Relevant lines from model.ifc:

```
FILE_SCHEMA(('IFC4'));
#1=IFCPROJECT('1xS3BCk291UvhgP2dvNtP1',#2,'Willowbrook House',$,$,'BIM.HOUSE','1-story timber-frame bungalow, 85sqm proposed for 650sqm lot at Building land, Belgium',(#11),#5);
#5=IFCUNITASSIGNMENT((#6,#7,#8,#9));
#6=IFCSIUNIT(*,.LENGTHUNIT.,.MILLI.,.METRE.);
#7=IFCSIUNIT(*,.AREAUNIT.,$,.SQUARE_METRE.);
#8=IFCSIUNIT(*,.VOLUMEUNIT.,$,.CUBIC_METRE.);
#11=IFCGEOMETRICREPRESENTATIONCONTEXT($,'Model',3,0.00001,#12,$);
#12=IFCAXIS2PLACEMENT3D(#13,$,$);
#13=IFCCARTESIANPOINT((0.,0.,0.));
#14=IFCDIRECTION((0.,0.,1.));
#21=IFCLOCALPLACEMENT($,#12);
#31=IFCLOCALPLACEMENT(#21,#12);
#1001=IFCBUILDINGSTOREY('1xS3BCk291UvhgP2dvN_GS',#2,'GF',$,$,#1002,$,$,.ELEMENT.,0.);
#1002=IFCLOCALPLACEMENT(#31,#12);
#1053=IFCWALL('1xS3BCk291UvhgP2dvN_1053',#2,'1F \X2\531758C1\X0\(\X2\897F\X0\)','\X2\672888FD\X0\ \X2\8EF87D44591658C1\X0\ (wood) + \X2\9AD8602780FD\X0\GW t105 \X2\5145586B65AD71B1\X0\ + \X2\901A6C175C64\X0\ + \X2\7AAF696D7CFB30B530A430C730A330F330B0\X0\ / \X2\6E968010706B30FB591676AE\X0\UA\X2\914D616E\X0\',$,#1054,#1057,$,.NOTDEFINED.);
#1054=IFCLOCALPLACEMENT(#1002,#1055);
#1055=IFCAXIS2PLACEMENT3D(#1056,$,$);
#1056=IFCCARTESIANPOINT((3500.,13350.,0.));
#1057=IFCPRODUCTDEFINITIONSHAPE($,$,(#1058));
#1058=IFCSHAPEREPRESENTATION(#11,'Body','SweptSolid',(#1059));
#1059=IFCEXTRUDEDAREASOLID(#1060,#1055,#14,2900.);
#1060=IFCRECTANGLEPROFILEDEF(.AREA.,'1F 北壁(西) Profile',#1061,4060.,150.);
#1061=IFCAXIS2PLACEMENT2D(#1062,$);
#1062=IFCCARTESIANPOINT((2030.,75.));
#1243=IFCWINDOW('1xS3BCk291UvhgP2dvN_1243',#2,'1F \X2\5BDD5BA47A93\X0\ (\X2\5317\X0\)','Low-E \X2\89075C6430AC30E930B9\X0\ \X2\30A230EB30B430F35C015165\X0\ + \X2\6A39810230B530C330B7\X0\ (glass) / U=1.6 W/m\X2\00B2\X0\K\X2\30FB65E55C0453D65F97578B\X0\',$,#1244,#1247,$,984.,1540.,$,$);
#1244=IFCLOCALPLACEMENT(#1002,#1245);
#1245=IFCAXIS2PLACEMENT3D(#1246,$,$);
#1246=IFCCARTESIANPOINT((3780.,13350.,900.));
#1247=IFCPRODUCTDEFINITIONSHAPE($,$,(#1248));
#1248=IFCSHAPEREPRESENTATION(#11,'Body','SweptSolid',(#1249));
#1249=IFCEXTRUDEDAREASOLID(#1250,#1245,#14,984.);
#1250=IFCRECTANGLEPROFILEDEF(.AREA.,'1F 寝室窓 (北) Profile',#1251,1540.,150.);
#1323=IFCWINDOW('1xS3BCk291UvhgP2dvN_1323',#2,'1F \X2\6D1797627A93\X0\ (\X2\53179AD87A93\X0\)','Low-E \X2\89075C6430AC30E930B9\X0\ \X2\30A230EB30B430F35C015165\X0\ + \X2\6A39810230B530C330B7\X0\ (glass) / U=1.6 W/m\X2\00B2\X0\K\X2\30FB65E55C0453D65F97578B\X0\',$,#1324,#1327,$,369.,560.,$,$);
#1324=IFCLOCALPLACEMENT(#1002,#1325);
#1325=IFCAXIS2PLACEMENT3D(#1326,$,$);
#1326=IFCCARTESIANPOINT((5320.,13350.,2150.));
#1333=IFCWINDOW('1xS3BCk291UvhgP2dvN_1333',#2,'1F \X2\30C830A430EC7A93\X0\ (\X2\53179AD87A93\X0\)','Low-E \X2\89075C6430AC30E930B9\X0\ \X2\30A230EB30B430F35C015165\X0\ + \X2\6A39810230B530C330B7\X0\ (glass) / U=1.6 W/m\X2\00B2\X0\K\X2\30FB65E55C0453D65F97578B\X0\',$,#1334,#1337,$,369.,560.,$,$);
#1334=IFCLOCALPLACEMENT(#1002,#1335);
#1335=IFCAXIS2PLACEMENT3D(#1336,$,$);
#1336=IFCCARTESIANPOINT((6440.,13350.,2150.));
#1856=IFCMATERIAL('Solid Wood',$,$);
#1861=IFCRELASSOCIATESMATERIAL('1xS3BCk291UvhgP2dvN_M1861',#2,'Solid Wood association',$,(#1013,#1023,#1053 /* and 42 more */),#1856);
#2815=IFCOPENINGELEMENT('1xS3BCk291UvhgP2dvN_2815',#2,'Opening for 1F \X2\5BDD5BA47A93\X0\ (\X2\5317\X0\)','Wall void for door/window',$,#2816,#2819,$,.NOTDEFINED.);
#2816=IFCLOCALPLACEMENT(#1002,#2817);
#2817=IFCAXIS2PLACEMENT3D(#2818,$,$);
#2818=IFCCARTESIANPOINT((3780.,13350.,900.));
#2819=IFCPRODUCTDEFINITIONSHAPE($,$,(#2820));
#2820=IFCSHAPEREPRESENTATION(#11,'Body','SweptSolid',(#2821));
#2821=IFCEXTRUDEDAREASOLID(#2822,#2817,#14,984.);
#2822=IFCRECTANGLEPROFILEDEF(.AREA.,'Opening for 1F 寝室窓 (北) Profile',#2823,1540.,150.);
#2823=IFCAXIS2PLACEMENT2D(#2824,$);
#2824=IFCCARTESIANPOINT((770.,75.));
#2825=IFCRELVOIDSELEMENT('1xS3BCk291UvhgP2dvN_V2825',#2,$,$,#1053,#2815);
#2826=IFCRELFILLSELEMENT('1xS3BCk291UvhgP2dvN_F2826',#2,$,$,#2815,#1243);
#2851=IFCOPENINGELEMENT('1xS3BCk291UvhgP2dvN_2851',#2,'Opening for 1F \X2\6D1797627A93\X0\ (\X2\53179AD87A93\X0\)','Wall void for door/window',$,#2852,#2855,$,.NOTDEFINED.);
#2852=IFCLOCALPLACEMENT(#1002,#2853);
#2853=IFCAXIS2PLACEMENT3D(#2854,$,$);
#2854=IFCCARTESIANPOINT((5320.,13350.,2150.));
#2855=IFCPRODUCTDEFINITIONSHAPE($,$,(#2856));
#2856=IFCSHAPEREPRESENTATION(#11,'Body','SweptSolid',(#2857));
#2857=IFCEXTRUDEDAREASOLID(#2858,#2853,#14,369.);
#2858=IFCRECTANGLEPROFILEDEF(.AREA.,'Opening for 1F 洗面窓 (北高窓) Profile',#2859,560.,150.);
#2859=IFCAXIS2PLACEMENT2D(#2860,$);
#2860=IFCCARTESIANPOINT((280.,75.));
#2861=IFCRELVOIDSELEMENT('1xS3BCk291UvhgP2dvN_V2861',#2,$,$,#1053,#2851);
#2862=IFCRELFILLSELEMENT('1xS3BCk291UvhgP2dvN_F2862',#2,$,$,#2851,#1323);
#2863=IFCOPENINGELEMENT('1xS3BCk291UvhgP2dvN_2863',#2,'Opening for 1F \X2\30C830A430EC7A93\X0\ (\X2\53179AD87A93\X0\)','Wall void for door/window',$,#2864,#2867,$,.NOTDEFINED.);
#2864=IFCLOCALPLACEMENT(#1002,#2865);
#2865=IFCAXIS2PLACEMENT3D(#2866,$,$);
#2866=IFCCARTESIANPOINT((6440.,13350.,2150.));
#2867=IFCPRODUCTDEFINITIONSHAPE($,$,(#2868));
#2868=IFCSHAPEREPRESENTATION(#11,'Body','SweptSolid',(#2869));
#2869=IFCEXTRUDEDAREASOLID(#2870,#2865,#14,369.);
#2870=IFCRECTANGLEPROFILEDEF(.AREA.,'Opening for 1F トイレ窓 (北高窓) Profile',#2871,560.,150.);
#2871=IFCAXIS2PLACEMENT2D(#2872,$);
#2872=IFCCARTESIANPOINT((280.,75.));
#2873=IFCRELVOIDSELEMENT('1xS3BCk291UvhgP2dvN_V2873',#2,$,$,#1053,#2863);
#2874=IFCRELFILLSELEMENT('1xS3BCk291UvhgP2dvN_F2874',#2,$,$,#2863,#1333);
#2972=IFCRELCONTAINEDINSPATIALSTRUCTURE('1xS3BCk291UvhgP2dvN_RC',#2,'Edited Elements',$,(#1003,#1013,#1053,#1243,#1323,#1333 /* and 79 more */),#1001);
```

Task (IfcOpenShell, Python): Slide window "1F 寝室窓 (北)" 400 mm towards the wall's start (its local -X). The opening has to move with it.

```python
import ifcopenshell
import ifcopenshell.api.geometry
import ifcopenshell.util.placement

model = ifcopenshell.open("model.ifc")

window = model.by_guid("1xS3BCk291UvhgP2dvN_1243")
opening = window.FillsVoids[0].RelatingOpeningElement
wall = opening.VoidsElements[0].RelatingBuildingElement

wall_matrix = ifcopenshell.util.placement.get_local_placement(wall.ObjectPlacement)
shift = wall_matrix[:3, 0] * -400.0
before = ifcopenshell.util.placement.get_local_placement(window.ObjectPlacement)[:3, 3].copy()

# The window is not placed relative to its opening, so move both.
for product in (opening, window):
    matrix = ifcopenshell.util.placement.get_local_placement(product.ObjectPlacement)
    matrix[:3, 3] += shift
    ifcopenshell.api.geometry.edit_object_placement(model, product=product, matrix=matrix, is_si=False)

after = ifcopenshell.util.placement.get_local_placement(window.ObjectPlacement)[:3, 3]
print("window moved by", (after - before).round(3) + 0.0)

model.write("model_edited.ifc")
```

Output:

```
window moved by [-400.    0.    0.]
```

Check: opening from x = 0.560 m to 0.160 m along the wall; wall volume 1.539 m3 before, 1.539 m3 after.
